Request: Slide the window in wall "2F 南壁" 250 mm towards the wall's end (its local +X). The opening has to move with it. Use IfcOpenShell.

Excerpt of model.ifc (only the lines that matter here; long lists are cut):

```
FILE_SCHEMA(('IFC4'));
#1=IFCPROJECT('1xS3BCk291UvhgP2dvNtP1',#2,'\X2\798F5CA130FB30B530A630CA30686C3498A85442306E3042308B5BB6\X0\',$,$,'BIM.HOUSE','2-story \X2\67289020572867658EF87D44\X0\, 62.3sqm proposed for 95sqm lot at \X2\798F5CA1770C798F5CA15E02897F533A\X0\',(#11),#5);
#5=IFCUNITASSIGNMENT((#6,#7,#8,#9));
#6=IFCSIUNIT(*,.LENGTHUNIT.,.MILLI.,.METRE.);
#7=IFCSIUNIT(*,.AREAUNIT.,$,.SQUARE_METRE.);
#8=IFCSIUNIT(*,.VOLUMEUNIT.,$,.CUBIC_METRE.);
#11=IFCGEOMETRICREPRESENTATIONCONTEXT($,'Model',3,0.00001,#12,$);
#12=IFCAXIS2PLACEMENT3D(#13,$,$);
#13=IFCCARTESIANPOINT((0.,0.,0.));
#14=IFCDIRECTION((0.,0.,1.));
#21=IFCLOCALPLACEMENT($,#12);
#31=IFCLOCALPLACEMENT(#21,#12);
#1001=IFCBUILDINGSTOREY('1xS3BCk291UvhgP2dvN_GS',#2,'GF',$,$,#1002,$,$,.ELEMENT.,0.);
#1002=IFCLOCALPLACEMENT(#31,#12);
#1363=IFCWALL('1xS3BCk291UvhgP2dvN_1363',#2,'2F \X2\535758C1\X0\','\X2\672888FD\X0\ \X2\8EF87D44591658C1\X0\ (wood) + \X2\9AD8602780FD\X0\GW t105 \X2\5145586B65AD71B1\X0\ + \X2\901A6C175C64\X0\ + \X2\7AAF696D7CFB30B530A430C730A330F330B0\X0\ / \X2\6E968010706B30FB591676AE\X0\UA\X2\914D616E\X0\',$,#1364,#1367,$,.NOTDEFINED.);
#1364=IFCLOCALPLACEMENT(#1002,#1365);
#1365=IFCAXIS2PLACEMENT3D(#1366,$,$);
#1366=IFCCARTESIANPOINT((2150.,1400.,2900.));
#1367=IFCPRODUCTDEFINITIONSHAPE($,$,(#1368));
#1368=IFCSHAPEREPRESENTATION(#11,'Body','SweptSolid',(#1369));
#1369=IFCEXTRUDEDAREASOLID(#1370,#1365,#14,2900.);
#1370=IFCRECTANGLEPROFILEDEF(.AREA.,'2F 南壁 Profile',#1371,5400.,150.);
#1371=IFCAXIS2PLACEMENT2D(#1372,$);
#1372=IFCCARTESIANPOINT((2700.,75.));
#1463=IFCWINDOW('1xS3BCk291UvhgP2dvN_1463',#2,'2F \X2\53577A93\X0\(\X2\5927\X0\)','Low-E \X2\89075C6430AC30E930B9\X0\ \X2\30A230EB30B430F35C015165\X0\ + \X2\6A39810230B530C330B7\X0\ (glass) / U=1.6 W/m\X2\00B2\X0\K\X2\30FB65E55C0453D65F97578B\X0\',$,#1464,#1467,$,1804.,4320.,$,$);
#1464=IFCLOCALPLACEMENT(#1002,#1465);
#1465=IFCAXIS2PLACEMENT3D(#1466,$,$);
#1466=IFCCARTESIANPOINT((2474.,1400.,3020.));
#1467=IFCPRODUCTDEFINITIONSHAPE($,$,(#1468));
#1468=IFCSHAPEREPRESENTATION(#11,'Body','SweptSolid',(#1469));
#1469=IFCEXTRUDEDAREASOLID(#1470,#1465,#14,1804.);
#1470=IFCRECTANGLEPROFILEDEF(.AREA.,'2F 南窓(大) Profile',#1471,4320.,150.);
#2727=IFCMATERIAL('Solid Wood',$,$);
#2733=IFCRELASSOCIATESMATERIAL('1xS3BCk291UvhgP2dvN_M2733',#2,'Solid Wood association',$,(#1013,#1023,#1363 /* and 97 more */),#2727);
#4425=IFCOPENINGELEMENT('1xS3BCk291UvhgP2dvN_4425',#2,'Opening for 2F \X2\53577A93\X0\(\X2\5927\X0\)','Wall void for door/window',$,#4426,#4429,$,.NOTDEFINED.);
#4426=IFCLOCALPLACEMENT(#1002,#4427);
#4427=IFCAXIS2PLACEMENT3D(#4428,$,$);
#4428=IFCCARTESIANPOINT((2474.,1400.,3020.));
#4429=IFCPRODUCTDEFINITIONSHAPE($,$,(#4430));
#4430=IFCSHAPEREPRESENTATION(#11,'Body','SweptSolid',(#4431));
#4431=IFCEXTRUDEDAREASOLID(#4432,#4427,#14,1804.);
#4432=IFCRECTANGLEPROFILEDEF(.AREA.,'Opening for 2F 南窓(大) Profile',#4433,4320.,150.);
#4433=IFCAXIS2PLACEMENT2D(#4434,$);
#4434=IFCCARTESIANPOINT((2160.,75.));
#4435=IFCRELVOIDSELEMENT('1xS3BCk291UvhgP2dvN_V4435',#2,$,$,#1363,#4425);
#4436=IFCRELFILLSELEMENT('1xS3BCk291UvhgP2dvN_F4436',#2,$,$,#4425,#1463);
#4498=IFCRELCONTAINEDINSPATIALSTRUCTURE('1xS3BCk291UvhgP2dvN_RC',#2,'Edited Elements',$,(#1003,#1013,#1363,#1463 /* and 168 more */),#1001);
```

```python
import ifcopenshell
import ifcopenshell.api.geometry
import ifcopenshell.util.placement
import ifcopenshell.util.unit

model = ifcopenshell.open("model.ifc")
unit_scale = ifcopenshell.util.unit.calculate_unit_scale(model)

window = model.by_id(1463)
opening = window.FillsVoids[0].RelatingOpeningElement
wall = opening.VoidsElements[0].RelatingBuildingElement

wall_matrix = ifcopenshell.util.placement.get_local_placement(wall.ObjectPlacement)
shift = wall_matrix[:3, 0] * 0.25 / unit_scale
before = ifcopenshell.util.placement.get_local_placement(window.ObjectPlacement)[:3, 3].copy()

# The window is not placed relative to its opening, so move both.
for product in (opening, window):
    matrix = ifcopenshell.util.placement.get_local_placement(product.ObjectPlacement)
    matrix[:3, 3] += shift
    ifcopenshell.api.geometry.edit_object_placement(model, product=product, matrix=matrix, is_si=False)

after = ifcopenshell.util.placement.get_local_placement(window.ObjectPlacement)[:3, 3]
print("window moved by", (after - before).round(3) + 0.0)

model.write("model_rev.ifc")
```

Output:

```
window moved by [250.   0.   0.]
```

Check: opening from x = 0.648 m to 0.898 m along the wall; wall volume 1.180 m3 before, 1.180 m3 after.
